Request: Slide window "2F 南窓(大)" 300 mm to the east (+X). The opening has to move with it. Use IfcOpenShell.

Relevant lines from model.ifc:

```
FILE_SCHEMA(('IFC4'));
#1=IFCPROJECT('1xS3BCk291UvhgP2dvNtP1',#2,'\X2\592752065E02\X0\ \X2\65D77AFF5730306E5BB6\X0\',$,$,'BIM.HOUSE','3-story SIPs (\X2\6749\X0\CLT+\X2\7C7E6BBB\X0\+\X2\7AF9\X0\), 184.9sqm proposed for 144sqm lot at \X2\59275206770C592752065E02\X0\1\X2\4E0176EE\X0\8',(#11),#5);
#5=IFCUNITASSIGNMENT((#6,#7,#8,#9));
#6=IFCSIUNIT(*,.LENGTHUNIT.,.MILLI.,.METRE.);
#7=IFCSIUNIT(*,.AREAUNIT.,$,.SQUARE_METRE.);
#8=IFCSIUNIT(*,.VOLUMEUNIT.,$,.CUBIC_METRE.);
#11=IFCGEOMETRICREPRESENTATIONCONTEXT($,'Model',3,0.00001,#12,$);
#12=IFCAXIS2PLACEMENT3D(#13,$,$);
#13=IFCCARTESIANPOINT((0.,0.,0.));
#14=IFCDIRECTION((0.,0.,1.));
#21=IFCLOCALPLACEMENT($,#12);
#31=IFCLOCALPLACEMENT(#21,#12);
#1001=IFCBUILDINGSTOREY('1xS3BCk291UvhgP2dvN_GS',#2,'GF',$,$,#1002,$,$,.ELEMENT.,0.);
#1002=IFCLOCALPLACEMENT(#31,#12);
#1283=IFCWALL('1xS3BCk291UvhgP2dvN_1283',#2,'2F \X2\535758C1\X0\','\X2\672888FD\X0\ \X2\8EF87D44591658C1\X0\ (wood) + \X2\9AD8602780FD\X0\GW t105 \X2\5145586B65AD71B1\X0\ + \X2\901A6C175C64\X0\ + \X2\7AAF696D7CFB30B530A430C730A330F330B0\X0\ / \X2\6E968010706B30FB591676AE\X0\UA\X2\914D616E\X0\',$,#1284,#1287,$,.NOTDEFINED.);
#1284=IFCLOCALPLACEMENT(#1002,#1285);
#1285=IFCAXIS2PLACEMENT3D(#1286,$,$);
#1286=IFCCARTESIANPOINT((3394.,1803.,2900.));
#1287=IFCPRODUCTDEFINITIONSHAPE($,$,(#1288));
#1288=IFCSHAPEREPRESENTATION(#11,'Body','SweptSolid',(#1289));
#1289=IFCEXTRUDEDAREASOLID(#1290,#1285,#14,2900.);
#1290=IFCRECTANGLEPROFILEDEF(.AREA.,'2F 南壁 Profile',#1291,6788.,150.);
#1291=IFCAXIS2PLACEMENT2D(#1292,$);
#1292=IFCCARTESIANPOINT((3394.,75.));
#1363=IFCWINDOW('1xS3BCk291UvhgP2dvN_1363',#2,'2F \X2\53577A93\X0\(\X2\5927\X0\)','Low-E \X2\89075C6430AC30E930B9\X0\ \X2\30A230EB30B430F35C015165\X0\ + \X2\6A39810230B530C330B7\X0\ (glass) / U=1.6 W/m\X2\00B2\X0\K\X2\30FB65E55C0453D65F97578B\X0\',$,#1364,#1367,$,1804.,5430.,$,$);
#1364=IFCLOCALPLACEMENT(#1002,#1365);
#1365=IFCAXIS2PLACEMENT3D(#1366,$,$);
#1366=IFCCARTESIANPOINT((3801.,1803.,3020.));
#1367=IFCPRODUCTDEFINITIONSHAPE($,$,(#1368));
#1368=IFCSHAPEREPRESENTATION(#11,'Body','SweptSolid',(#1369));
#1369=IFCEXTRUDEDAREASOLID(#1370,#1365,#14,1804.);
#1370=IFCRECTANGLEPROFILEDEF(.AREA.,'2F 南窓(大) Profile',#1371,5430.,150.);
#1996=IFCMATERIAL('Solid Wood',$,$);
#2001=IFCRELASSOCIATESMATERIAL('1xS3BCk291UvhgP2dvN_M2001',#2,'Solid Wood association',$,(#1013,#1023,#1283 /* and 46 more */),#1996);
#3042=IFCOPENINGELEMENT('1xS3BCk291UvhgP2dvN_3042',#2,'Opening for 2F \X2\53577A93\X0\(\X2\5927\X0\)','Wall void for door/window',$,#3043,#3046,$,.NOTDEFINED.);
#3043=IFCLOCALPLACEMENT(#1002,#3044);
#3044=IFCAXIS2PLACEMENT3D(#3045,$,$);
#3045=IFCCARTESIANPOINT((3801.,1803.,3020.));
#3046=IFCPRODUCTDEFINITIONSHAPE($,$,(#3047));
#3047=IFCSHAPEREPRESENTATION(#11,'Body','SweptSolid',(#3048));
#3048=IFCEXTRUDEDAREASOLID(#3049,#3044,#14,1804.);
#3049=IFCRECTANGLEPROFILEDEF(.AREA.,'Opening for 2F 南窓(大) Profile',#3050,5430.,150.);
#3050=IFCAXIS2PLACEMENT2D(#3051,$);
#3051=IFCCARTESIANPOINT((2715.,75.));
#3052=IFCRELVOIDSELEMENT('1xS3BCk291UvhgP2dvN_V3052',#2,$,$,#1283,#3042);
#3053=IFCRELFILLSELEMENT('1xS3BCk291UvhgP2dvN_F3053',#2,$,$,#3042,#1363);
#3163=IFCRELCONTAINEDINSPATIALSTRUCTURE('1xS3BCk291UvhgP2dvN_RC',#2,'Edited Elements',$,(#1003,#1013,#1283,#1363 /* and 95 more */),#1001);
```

```python
import ifcopenshell
import ifcopenshell.api.geometry
import ifcopenshell.util.placement

model = ifcopenshell.open("model.ifc")

window = model.by_guid("1xS3BCk291UvhgP2dvN_1363")
opening = window.FillsVoids[0].RelatingOpeningElement
wall = opening.VoidsElements[0].RelatingBuildingElement

wall_matrix = ifcopenshell.util.placement.get_local_placement(wall.ObjectPlacement)
shift = wall_matrix[:3, 0] * 300.0
before = ifcopenshell.util.placement.get_local_placement(window.ObjectPlacement)[:3, 3].copy()

# The window is not placed relative to its opening, so move both.
for product in (opening, window):
    matrix = ifcopenshell.util.placement.get_local_placement(product.ObjectPlacement)
    matrix[:3, 3] += shift
    ifcopenshell.api.geometry.edit_object_placement(model, product=product, matrix=matrix, is_si=False)

after = ifcopenshell.util.placement.get_local_placement(window.ObjectPlacement)[:3, 3]
print("window moved by", (after - before).round(3) + 0.0)

model.write("model_v2.ifc")
```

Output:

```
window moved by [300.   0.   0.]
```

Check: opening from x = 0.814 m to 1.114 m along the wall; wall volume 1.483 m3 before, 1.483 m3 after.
